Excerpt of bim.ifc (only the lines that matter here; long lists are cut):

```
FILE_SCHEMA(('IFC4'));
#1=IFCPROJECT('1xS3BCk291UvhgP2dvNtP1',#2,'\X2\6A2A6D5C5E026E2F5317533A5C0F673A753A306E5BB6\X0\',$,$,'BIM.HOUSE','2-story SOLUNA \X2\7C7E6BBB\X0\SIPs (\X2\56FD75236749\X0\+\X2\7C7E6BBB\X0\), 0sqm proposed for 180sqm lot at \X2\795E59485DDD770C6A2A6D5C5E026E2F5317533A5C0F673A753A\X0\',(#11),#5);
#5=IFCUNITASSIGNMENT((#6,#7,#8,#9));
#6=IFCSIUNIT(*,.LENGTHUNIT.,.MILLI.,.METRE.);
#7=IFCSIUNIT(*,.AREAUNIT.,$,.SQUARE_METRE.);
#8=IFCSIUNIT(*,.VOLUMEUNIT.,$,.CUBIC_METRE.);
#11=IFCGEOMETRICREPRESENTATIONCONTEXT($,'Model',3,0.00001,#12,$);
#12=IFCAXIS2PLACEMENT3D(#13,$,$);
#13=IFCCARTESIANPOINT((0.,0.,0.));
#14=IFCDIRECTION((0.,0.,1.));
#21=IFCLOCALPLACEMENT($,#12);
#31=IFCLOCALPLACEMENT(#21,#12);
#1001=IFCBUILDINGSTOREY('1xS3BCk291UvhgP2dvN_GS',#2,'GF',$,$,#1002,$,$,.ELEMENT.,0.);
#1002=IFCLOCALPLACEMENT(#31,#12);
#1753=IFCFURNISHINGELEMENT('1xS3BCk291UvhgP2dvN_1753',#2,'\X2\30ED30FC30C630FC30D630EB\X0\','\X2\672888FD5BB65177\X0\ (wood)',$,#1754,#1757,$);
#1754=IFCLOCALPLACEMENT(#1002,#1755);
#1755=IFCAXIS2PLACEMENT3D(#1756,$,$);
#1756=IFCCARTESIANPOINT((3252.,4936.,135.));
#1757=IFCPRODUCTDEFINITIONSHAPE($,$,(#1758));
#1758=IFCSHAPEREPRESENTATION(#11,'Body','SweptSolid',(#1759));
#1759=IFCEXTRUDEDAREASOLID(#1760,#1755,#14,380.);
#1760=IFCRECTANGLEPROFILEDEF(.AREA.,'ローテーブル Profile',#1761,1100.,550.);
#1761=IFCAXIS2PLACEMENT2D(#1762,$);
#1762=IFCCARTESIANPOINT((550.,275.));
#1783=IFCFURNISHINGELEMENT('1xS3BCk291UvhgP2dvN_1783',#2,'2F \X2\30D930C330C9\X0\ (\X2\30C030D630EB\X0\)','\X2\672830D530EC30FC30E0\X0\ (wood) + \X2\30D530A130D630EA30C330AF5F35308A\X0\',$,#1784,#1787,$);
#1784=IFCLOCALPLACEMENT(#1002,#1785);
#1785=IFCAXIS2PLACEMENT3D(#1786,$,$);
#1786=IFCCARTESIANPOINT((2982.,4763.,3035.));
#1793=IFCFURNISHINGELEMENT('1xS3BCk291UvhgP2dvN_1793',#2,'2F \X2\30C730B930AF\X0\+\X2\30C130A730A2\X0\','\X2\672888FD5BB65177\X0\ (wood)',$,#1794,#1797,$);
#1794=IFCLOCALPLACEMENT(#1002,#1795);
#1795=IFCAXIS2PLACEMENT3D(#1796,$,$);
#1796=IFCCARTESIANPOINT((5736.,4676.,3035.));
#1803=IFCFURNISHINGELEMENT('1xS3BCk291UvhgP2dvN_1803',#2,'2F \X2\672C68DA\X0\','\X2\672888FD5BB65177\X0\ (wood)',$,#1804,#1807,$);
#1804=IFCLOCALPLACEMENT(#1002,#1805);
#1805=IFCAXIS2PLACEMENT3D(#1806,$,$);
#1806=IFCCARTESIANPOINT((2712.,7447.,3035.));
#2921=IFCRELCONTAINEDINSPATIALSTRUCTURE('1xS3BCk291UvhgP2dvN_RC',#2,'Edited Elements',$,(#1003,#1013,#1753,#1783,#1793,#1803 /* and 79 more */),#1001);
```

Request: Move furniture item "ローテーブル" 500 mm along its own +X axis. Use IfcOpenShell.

```python
import ifcopenshell
import ifcopenshell.api.geometry
import ifcopenshell.util.placement
import ifcopenshell.util.unit

model = ifcopenshell.open("bim.ifc")
unit_scale = ifcopenshell.util.unit.calculate_unit_scale(model)

item = model.by_guid("1xS3BCk291UvhgP2dvN_1753")
matrix = ifcopenshell.util.placement.get_local_placement(item.ObjectPlacement)
matrix[:3, 3] += matrix[:3, 0] * 0.5 / unit_scale
ifcopenshell.api.geometry.edit_object_placement(model, product=item, matrix=matrix, is_si=False)

print(ifcopenshell.util.placement.get_local_placement(item.ObjectPlacement).round(3) + 0.0)

model.write("bim-out.ifc")
```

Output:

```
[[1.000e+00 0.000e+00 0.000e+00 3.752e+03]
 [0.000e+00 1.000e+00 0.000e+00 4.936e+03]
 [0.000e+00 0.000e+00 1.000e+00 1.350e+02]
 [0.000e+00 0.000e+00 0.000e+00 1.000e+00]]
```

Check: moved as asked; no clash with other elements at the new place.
